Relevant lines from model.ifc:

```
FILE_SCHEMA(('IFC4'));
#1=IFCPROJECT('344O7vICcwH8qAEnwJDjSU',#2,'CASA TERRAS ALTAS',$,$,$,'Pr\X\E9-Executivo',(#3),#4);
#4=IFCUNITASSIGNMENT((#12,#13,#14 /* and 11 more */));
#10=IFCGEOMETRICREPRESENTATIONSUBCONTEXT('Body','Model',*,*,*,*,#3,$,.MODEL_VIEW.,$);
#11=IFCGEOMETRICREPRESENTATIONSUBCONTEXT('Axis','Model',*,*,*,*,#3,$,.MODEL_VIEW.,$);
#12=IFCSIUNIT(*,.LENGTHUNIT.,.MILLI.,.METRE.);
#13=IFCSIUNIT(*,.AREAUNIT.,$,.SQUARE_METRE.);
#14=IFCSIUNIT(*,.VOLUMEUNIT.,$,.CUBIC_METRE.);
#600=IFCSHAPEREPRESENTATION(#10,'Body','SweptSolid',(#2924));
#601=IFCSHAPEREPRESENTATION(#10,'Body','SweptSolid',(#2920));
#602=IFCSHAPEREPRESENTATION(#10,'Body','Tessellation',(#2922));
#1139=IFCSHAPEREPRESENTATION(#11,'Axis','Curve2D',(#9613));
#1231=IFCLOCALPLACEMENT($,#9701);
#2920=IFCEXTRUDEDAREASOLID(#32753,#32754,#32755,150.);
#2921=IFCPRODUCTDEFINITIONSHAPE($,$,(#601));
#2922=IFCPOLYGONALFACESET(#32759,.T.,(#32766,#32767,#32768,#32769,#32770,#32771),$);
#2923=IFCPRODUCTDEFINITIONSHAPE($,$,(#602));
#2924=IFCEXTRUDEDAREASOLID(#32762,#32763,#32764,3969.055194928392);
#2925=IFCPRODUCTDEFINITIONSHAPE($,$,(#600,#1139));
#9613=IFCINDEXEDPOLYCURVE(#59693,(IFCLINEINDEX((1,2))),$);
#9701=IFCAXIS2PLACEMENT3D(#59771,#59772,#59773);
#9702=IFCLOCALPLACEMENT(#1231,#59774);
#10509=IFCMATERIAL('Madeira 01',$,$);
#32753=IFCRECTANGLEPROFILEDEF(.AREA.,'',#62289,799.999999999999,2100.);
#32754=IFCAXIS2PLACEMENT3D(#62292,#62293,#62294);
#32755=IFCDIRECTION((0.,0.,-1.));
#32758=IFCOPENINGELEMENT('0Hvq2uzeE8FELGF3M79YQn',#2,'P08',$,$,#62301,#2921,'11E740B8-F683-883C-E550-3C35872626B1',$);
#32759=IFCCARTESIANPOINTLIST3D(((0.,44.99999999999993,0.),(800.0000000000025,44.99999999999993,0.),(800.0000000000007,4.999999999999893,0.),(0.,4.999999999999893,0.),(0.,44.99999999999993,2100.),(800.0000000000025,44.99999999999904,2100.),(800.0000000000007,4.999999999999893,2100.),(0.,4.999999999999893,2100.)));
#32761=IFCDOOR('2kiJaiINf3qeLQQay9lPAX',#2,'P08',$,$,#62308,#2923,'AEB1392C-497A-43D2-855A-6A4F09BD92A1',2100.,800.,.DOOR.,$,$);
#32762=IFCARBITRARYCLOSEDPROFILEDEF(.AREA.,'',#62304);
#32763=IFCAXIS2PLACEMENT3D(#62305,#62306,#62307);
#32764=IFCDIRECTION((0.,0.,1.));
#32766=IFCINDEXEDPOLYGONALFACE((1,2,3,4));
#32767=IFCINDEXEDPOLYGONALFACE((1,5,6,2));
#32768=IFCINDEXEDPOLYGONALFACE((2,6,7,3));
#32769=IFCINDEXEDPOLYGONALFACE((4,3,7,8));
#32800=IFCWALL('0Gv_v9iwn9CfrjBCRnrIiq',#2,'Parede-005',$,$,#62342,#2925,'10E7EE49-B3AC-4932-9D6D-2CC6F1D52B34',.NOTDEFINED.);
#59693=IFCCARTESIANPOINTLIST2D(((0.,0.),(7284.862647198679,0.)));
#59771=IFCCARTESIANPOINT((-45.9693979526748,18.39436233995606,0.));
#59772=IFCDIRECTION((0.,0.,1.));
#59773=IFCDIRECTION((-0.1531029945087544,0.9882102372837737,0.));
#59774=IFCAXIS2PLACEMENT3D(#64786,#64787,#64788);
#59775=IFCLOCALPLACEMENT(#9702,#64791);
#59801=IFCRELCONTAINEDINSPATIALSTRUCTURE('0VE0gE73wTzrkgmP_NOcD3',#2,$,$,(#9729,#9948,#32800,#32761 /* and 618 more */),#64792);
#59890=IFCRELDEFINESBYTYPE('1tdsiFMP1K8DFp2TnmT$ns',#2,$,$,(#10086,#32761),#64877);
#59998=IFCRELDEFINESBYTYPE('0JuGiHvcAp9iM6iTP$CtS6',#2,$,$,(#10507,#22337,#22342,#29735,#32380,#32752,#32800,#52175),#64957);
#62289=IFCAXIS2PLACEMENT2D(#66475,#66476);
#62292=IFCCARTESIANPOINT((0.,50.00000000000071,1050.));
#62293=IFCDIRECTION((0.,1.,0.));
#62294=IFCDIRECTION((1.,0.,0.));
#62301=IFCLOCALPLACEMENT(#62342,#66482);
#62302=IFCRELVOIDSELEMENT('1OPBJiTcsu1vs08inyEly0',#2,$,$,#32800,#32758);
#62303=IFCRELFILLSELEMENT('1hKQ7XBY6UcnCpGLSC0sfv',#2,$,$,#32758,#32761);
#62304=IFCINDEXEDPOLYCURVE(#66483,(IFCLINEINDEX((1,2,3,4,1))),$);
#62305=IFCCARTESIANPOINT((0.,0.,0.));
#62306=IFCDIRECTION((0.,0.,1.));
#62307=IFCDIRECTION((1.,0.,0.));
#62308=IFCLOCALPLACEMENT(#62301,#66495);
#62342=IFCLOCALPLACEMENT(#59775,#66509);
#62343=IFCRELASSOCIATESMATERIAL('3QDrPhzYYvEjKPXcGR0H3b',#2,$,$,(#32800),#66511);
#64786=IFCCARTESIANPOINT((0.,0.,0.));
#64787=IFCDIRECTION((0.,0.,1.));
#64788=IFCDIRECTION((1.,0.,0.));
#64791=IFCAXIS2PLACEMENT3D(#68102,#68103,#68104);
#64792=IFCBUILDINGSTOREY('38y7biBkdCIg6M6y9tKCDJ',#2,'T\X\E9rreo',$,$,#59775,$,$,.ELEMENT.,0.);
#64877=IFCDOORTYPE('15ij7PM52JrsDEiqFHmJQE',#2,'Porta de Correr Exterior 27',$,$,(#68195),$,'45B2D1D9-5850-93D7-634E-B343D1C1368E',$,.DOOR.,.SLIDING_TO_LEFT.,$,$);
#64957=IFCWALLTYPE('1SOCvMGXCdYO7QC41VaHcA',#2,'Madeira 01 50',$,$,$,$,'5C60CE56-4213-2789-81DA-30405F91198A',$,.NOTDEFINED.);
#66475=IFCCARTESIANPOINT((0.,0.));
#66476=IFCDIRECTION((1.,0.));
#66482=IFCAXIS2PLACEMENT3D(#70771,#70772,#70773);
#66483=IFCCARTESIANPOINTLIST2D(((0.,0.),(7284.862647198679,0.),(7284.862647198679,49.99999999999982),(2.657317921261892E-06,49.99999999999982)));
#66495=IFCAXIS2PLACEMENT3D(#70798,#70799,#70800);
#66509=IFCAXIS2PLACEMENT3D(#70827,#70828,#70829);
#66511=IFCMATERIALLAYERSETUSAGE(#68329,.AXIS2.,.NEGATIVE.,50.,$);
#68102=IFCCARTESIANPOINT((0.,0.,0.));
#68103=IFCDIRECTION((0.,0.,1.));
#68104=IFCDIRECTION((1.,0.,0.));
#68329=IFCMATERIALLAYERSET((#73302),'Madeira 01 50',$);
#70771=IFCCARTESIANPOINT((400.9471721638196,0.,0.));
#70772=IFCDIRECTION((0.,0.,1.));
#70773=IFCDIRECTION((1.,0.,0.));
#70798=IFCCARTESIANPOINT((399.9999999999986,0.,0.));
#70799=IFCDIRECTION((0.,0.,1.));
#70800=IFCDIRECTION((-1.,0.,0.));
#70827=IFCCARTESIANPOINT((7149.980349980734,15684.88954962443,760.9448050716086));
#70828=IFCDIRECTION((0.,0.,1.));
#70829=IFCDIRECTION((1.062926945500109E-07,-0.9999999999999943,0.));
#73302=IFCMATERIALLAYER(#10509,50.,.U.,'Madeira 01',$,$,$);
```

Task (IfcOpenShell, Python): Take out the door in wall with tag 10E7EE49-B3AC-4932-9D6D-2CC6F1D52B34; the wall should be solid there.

```python
import ifcopenshell
import ifcopenshell.api.feature
import ifcopenshell.api.root
import ifcopenshell.geom
import ifcopenshell.util.shape

model = ifcopenshell.open("model.ifc")
settings = ifcopenshell.geom.settings()


def volume(element):
    """Net volume in cubic metres, openings subtracted."""
    shape = ifcopenshell.geom.create_shape(settings, element)
    return ifcopenshell.util.shape.get_volume(shape.geometry)


door = model.by_id(32761)
opening = door.FillsVoids[0].RelatingOpeningElement
wall = opening.VoidsElements[0].RelatingBuildingElement
before = volume(wall)

ifcopenshell.api.root.remove_product(model, product=door)
ifcopenshell.api.feature.remove_feature(model, feature=opening)

after = volume(wall)

print(f"wall volume {before:.3f} -> {after:.3f} m3")

model.write("model_edited.ifc")
```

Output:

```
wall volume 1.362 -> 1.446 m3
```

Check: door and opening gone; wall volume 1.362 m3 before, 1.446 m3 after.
